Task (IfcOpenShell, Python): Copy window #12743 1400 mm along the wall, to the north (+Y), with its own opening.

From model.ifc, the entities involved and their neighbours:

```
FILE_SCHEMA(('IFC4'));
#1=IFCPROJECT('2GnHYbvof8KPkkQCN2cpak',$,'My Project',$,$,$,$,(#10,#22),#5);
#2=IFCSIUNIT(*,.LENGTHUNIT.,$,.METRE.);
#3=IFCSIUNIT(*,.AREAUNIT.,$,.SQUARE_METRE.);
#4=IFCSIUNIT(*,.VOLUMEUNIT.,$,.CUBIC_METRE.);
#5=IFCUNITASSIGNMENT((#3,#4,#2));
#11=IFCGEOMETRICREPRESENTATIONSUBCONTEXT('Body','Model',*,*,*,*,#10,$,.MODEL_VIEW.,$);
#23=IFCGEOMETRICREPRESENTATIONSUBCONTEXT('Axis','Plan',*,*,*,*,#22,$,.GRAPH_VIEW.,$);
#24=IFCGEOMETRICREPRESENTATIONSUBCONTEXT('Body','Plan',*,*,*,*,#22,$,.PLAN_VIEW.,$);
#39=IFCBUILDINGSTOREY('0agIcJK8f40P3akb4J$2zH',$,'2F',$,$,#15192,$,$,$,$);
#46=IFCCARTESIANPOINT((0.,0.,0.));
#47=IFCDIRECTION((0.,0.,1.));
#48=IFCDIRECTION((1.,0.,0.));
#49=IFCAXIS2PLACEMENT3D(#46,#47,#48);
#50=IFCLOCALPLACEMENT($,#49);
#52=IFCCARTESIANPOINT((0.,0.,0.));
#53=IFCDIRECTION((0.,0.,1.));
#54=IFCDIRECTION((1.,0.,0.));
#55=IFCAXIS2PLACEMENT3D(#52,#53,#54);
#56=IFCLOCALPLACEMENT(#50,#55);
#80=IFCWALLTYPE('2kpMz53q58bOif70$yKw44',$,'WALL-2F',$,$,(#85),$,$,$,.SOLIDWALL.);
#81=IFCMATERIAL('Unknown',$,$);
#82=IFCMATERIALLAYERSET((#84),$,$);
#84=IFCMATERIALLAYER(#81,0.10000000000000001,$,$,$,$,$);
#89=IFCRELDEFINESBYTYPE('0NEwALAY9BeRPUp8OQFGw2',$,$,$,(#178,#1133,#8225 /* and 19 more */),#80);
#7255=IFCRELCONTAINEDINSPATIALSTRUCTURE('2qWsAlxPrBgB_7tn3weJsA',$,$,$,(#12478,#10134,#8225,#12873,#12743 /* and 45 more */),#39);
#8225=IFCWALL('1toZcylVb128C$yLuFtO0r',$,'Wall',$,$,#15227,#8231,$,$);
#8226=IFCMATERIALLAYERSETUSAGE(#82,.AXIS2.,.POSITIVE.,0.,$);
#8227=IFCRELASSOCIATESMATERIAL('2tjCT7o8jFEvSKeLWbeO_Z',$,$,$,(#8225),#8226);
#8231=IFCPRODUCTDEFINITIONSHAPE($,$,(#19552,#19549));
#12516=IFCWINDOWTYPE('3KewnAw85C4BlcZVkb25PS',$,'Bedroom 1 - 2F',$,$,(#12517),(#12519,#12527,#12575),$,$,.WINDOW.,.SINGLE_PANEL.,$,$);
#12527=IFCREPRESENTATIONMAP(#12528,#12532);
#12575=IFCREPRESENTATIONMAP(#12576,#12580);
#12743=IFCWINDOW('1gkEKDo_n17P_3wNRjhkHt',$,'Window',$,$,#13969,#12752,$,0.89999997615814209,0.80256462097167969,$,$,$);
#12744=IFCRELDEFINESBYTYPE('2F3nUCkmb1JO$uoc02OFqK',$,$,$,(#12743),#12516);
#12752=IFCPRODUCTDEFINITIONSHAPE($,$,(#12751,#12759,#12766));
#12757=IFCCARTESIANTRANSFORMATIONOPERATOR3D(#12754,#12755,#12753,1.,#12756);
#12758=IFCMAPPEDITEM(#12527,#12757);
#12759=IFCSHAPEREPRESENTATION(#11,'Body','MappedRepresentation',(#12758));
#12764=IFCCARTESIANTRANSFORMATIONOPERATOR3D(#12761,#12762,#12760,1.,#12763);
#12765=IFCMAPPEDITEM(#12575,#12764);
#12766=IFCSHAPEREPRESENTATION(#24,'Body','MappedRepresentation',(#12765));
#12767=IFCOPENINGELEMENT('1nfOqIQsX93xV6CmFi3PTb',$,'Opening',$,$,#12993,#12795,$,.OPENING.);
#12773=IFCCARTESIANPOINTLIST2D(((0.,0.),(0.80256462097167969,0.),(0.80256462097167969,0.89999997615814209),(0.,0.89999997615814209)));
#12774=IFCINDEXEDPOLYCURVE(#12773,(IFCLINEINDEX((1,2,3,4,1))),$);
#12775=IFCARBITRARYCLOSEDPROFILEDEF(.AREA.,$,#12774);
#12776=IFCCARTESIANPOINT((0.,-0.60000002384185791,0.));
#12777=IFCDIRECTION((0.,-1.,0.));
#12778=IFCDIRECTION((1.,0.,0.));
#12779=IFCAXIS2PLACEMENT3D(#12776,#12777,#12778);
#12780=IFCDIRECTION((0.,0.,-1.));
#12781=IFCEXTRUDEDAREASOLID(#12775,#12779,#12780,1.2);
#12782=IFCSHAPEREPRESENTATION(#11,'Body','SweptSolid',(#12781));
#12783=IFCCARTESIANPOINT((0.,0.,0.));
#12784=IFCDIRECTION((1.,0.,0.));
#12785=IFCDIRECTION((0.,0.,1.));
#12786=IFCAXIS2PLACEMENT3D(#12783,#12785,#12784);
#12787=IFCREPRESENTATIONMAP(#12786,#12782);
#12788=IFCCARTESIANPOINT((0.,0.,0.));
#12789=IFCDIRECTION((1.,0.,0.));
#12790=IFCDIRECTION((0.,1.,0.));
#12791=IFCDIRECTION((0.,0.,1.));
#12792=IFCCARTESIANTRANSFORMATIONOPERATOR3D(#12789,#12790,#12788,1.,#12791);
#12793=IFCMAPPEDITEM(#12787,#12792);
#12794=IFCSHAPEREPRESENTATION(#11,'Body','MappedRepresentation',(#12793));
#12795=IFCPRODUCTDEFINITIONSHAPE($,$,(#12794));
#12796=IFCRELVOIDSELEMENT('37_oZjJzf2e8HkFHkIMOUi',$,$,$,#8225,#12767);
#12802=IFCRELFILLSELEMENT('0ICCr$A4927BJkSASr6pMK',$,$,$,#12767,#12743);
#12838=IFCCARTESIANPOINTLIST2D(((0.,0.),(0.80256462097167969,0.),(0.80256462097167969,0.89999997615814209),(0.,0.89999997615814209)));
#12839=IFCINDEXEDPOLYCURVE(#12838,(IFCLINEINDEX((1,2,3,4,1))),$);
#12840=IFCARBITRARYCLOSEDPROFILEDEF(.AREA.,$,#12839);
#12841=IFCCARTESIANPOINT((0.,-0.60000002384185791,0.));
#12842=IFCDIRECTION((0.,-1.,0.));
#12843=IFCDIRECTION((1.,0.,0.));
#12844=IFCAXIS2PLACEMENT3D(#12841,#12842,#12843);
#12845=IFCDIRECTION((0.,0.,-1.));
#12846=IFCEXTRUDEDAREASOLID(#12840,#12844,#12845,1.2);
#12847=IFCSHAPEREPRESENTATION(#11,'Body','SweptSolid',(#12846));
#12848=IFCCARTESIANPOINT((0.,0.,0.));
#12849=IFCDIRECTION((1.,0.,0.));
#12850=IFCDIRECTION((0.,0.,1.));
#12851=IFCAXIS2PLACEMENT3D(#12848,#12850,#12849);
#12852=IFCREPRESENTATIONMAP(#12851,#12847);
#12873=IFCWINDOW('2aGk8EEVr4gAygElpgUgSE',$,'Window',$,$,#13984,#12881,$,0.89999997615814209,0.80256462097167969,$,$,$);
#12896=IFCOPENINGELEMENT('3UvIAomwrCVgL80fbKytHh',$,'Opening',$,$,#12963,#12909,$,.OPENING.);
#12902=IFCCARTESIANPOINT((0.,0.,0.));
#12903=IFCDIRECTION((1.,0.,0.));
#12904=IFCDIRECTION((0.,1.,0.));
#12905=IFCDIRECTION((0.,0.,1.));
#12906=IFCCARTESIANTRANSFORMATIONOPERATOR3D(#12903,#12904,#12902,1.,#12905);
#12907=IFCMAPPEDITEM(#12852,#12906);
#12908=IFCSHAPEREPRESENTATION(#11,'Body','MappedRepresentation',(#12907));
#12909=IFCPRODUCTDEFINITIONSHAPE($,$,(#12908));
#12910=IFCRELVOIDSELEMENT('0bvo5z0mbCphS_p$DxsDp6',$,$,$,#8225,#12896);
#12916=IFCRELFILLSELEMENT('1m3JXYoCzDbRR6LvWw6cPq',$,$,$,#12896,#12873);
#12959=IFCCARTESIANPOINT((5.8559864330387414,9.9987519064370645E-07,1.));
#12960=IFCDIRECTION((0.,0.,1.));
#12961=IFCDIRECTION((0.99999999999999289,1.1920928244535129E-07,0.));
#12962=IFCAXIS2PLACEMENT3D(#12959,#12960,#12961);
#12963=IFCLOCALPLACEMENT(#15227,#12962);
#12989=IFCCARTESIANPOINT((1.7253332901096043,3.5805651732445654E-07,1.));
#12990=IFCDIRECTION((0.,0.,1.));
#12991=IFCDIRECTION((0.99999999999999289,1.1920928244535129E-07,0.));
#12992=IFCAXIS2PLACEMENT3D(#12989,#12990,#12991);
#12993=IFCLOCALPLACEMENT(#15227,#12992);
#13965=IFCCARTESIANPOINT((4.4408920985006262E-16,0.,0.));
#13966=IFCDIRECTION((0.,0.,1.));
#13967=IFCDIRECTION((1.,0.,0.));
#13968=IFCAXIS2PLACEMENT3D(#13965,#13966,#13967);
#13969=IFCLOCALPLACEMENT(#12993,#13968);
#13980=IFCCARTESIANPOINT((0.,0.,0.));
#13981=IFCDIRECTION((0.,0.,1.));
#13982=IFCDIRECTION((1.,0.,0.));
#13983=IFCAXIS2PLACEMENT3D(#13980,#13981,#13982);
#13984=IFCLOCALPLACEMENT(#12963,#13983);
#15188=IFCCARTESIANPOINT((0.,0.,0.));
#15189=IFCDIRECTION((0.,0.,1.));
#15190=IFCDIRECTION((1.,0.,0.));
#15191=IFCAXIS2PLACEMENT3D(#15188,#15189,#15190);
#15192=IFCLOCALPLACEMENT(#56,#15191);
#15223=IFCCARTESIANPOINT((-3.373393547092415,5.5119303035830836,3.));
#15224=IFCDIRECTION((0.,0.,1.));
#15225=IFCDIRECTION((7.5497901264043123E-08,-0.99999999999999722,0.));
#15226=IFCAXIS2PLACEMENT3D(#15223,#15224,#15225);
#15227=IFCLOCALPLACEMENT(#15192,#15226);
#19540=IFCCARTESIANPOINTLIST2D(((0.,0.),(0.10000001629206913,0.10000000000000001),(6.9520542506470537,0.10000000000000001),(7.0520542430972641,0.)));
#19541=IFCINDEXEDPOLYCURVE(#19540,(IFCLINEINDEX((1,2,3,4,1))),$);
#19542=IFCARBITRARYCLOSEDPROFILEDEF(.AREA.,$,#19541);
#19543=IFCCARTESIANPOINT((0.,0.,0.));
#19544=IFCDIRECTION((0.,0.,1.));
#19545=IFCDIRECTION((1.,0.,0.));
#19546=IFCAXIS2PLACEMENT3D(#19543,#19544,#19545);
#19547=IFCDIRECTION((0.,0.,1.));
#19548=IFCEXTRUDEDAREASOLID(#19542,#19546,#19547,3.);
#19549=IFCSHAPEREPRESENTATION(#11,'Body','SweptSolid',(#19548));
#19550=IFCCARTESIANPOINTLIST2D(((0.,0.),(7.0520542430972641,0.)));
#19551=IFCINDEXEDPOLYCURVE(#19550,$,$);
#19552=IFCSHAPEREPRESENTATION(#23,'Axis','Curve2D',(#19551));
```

```python
import ifcopenshell
import ifcopenshell.api.feature
import ifcopenshell.api.geometry
import ifcopenshell.api.root
import ifcopenshell.geom
import ifcopenshell.util.element
import ifcopenshell.util.placement
import ifcopenshell.util.shape
import ifcopenshell.util.unit

model = ifcopenshell.open("model.ifc")
unit_scale = ifcopenshell.util.unit.calculate_unit_scale(model)
settings = ifcopenshell.geom.settings()


def volume(element):
    """Net volume in cubic metres, openings subtracted."""
    shape = ifcopenshell.geom.create_shape(settings, element)
    return ifcopenshell.util.shape.get_volume(shape.geometry)


window = model.by_guid("1gkEKDo_n17P_3wNRjhkHt")
opening = window.FillsVoids[0].RelatingOpeningElement
wall = opening.VoidsElements[0].RelatingBuildingElement
before = volume(wall)
shift = ifcopenshell.util.placement.get_local_placement(wall.ObjectPlacement)[:3, 0] * -1.4 / unit_scale

# copy_class copies the void relationship, type, container and properties, but no geometry.
new_opening = ifcopenshell.api.root.copy_class(model, product=opening)
new_opening.Representation = ifcopenshell.util.element.copy_deep(
    model, opening.Representation, exclude=["IfcGeometricRepresentationContext", "IfcRepresentationMap"]
)
new_window = ifcopenshell.api.root.copy_class(model, product=window)
new_window.Representation = ifcopenshell.util.element.copy_deep(
    model, window.Representation, exclude=["IfcGeometricRepresentationContext", "IfcRepresentationMap"]
)
ifcopenshell.api.feature.add_filling(model, opening=new_opening, element=new_window)

for old, new in ((opening, new_opening), (window, new_window)):
    matrix = ifcopenshell.util.placement.get_local_placement(old.ObjectPlacement)
    matrix[:3, 3] += shift
    ifcopenshell.api.geometry.edit_object_placement(model, product=new, matrix=matrix, is_si=False)

after = volume(wall)

print(f"wall volume {before:.3f} -> {after:.3f} m3")

model.write("model-out.ifc")
```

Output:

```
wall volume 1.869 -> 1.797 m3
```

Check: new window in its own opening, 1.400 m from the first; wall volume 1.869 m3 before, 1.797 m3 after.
